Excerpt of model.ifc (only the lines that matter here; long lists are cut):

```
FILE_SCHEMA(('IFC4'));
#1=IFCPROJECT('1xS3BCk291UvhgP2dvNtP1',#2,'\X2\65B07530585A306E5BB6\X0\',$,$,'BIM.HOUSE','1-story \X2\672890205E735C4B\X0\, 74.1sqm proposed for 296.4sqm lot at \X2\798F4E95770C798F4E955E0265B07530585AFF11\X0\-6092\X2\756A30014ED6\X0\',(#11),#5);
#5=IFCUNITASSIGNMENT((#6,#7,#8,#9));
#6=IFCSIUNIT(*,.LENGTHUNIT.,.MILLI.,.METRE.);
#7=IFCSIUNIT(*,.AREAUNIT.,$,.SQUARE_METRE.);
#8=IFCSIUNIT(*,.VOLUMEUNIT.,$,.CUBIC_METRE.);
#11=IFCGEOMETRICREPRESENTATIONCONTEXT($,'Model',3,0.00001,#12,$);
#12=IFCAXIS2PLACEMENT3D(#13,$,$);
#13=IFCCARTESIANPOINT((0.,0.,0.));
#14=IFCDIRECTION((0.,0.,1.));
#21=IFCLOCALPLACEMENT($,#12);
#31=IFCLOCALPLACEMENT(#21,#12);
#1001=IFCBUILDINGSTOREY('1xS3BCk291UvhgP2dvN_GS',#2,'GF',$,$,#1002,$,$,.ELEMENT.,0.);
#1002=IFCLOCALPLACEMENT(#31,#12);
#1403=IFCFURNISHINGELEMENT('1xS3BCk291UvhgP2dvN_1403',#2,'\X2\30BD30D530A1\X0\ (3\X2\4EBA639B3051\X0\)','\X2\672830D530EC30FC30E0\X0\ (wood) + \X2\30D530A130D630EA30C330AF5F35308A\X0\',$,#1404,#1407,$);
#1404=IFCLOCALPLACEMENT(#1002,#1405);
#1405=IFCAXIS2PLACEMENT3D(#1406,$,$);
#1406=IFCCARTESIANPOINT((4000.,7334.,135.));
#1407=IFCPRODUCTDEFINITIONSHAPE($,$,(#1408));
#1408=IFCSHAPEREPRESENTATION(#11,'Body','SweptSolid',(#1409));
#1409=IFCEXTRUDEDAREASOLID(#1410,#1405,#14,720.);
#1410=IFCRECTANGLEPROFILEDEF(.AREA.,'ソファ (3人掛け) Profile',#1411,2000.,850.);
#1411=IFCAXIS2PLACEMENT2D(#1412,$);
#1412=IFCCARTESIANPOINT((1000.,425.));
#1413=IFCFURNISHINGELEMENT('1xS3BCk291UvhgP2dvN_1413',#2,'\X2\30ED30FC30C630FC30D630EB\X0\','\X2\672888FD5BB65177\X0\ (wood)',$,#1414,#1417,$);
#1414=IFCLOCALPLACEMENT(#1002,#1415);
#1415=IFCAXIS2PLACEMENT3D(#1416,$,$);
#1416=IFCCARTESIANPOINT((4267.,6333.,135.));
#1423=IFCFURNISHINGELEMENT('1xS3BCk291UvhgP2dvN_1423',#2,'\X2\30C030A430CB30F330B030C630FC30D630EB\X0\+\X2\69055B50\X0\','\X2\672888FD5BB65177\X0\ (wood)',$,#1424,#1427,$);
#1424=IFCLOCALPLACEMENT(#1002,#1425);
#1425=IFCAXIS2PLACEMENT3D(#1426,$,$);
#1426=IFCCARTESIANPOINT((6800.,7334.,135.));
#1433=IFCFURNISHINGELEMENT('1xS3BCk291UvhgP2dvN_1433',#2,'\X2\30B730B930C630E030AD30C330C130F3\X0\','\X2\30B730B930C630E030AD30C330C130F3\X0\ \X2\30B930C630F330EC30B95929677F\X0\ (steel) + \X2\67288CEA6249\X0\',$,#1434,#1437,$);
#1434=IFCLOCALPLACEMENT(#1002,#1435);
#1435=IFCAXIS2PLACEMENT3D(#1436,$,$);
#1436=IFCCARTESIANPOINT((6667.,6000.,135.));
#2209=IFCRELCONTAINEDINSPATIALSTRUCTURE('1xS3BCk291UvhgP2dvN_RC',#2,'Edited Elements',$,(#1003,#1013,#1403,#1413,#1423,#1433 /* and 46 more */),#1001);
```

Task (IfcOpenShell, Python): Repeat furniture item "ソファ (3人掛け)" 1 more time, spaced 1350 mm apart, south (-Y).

```python
import numpy as np
import ifcopenshell
import ifcopenshell.api.geometry
import ifcopenshell.api.root
import ifcopenshell.util.element
import ifcopenshell.util.placement

model = ifcopenshell.open("model.ifc")


def reuse_history(source, copy):
    """copy_class also copies each property set's owner history, people and application; keep the originals."""
    for rel in copy.IsDefinedBy:
        if rel.is_a("IfcRelDefinesByProperties") and (history := rel.RelatingPropertyDefinition.OwnerHistory):
            rel.RelatingPropertyDefinition.OwnerHistory = source.OwnerHistory
            ifcopenshell.util.element.remove_deep2(model, history)


source = model.by_guid("1xS3BCk291UvhgP2dvN_1403")
base = ifcopenshell.util.placement.get_local_placement(source.ObjectPlacement)
step = np.array([0.0, -1.0, 0.0]) * 1350.0

for i in range(1, 2):
    copy = ifcopenshell.api.root.copy_class(model, product=source)
    copy.Representation = ifcopenshell.util.element.copy_deep(
        model, source.Representation, exclude=["IfcGeometricRepresentationContext", "IfcRepresentationMap"]
    )
    reuse_history(source, copy)
    matrix = base.copy()
    matrix[:3, 3] += i * step
    print("added at", matrix[:3, 3].round(3) + 0.0)
    ifcopenshell.api.geometry.edit_object_placement(model, product=copy, matrix=matrix, is_si=False)

model.write("model-out.ifc")
```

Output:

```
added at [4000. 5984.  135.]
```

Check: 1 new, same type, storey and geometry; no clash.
